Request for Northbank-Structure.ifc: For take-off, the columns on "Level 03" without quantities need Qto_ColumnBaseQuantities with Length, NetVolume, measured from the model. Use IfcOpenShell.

First a look at what the model holds.

```python
import ifcopenshell
import ifcopenshell.util.element
import ifcopenshell.util.unit

model = ifcopenshell.open("Northbank-Structure.ifc")
print(model.schema)
for unit_type in ("LENGTHUNIT", "AREAUNIT", "VOLUMEUNIT"):
    print(unit_type, ifcopenshell.util.unit.calculate_unit_scale(model, unit_type))
storey = next(s for s in model.by_type("IfcBuildingStorey") if s.Name == "Level 03")
columns = [e for e in ifcopenshell.util.element.get_decomposition(storey) if e.is_a("IfcColumn")]
for e in sorted(columns, key=lambda e: e.id()):
    print(e.id(), e.is_a(), e.Name, list(ifcopenshell.util.element.get_psets(e, qtos_only=True)), sep=" | ")
```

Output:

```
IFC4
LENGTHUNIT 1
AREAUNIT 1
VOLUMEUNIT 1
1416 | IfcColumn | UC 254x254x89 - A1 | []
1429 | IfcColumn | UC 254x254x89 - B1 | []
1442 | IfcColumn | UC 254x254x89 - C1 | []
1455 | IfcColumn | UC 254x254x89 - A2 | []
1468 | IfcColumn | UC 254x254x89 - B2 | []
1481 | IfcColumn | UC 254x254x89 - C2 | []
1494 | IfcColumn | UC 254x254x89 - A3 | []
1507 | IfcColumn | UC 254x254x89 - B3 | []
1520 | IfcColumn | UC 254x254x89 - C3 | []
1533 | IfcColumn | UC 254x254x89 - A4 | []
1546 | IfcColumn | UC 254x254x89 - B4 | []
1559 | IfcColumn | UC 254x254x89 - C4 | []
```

```python
import ifcopenshell
import ifcopenshell.api.pset
import ifcopenshell.geom
import ifcopenshell.util.element
import ifcopenshell.util.shape
import ifcopenshell.util.unit

model = ifcopenshell.open("Northbank-Structure.ifc")
unit_scale = ifcopenshell.util.unit.calculate_unit_scale(model)
volume_scale = ifcopenshell.util.unit.calculate_unit_scale(model, "VOLUMEUNIT")
settings = ifcopenshell.geom.settings()

storey = next(s for s in model.by_type("IfcBuildingStorey") if s.Name == "Level 03")
columns = [e for e in ifcopenshell.util.element.get_decomposition(storey) if e.is_a("IfcColumn")]

for e in sorted(columns, key=lambda e: e.id()):
    if ifcopenshell.util.element.get_psets(e, qtos_only=True, should_inherit=False):
        continue
    # Geometry comes back in metres, in the element's own axes.
    shape = ifcopenshell.geom.create_shape(settings, e)
    values = {
        "Length": ifcopenshell.util.shape.get_z(shape.geometry) / unit_scale,
        "NetVolume": ifcopenshell.util.shape.get_volume(shape.geometry) / volume_scale,
    }
    qto = ifcopenshell.api.pset.add_qto(model, product=e, name="Qto_ColumnBaseQuantities")
    ifcopenshell.api.pset.edit_qto(model, qto=qto, properties=values)
    print(e.id(), {k: round(v, 3) for k, v in values.items()})

model.write("Northbank-Structure-out.ifc")
```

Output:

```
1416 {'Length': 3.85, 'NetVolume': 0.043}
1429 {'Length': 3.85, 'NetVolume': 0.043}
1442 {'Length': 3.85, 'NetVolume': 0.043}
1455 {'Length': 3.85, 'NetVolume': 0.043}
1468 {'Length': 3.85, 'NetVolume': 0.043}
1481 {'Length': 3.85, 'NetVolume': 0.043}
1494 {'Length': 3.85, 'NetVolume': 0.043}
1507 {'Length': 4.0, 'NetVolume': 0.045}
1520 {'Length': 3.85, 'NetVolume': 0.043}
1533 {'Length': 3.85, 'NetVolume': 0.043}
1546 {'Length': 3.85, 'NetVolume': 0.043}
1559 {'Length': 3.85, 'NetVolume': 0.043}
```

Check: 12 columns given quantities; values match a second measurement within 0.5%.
